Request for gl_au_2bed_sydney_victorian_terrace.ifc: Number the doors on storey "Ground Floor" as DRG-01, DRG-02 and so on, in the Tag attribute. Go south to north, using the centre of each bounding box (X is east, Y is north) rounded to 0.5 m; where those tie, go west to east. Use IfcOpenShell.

First a look at what the model holds.

```python
import ifcopenshell
import ifcopenshell.util.element
import ifcopenshell.util.placement

model = ifcopenshell.open("gl_au_2bed_sydney_victorian_terrace.ifc")
print(model.schema)
storey = next(s for s in model.by_type("IfcBuildingStorey") if s.Name == "Ground Floor")
doors = [e for e in ifcopenshell.util.element.get_decomposition(storey) if e.is_a("IfcDoor")]
for e in sorted(doors, key=lambda e: e.id()):
    origin = ifcopenshell.util.placement.get_local_placement(e.ObjectPlacement)[:3, 3]
    print(e.id(), e.Tag, e.Name, origin.round(2) + 0.0, sep=" | ")
```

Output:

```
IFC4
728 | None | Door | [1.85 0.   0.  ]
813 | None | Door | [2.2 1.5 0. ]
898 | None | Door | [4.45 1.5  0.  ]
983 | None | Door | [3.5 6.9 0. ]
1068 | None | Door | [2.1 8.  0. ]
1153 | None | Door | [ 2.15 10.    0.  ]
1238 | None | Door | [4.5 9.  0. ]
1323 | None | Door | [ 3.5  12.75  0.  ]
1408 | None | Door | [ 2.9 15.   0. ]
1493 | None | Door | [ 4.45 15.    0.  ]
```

```python
import ifcopenshell
import ifcopenshell.geom
import ifcopenshell.util.element
import ifcopenshell.util.shape

model = ifcopenshell.open("gl_au_2bed_sydney_victorian_terrace.ifc")
settings = ifcopenshell.geom.settings()
settings.set("use-world-coords", True)


def centre(element):
    shape = ifcopenshell.geom.create_shape(settings, element)
    return ifcopenshell.util.shape.get_bbox_centroid(shape.geometry)


storey = next(s for s in model.by_type("IfcBuildingStorey") if s.Name == "Ground Floor")
doors = [e for e in ifcopenshell.util.element.get_decomposition(storey) if e.is_a("IfcDoor")]

# Insertion points can sit at a corner or the storey origin, so sort by the geometry (in metres).
centres = {e: centre(e) for e in doors}
doors.sort(key=lambda e: (round(centres[e][1] / 0.5), centres[e][0]))

for i, e in enumerate(doors, start=1):
    number = f"DRG-{i:02d}"
    e.Tag = number
    print(e.id(), number)

model.write("gl_au_2bed_sydney_victorian_terrace-out.ifc")
```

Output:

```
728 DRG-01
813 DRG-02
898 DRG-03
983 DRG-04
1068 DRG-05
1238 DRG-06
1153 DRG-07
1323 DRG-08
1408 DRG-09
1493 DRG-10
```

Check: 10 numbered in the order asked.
